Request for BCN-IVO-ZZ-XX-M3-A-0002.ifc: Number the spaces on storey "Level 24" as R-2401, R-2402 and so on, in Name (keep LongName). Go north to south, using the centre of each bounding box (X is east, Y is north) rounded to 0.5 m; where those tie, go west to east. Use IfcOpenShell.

First a look at what the model holds.

```python
import ifcopenshell
import ifcopenshell.util.element
import ifcopenshell.util.placement

model = ifcopenshell.open("BCN-IVO-ZZ-XX-M3-A-0002.ifc")
print(model.schema)
storey = next(s for s in model.by_type("IfcBuildingStorey") if s.Name == "Level 24")
spaces = [e for e in ifcopenshell.util.element.get_decomposition(storey) if e.is_a("IfcSpace")]
for e in sorted(spaces, key=lambda e: e.id()):
    origin = ifcopenshell.util.placement.get_local_placement(e.ObjectPlacement)[:3, 3]
    print(e.id(), e.Name, e.LongName, origin.round(2) + 0.0, sep=" | ")
```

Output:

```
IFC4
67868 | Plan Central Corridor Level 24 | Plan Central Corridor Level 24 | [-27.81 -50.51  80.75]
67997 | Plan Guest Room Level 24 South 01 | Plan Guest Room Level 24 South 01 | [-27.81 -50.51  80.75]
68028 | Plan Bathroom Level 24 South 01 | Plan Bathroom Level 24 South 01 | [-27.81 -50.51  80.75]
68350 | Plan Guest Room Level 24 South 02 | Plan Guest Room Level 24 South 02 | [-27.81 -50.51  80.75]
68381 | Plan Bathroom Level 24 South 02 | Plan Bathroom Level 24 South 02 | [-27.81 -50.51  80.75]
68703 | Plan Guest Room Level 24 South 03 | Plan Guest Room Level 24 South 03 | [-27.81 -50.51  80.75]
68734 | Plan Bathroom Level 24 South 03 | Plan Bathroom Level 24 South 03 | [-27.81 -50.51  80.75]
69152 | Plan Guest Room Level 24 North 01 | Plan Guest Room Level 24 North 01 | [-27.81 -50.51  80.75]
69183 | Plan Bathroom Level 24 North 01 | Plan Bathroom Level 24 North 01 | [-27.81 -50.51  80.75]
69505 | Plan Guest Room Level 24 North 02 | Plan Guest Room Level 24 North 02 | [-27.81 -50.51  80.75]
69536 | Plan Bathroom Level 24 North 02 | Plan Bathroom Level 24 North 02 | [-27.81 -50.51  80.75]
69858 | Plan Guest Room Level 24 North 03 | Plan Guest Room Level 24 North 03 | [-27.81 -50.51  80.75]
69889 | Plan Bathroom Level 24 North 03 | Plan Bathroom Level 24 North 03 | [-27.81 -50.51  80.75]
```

```python
import ifcopenshell
import ifcopenshell.geom
import ifcopenshell.util.element
import ifcopenshell.util.shape

model = ifcopenshell.open("BCN-IVO-ZZ-XX-M3-A-0002.ifc")
settings = ifcopenshell.geom.settings()
settings.set("use-world-coords", True)


def centre(element):
    shape = ifcopenshell.geom.create_shape(settings, element)
    return ifcopenshell.util.shape.get_bbox_centroid(shape.geometry)


storey = next(s for s in model.by_type("IfcBuildingStorey") if s.Name == "Level 24")
spaces = [e for e in ifcopenshell.util.element.get_decomposition(storey) if e.is_a("IfcSpace")]

# Insertion points can sit at a corner or the storey origin, so sort by the geometry (in metres).
centres = {e: centre(e) for e in spaces}
spaces.sort(key=lambda e: (-round(centres[e][1] / 0.5), centres[e][0]))

for i, e in enumerate(spaces, start=1):
    number = f"R-24{i:02d}"
    e.Name = number
    print(e.id(), number)

model.write("BCN-IVO-ZZ-XX-M3-A-0002-out.ifc")
```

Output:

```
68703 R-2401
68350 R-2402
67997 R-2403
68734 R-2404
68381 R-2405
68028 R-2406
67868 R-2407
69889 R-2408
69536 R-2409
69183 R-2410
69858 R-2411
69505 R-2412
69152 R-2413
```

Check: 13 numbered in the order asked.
